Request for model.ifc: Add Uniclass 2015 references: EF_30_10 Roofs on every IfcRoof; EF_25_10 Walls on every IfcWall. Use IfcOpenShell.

First a look at what the model holds.

```python
import ifcopenshell

model = ifcopenshell.open("model.ifc")
print(model.schema)
print("classifications:", [c.Name for c in model.by_type("IfcClassification")])
for ifc_class in ("IfcDoor", "IfcRoof", "IfcStair", "IfcWall", "IfcWindow"):
    print(ifc_class, len(model.by_type(ifc_class)))
```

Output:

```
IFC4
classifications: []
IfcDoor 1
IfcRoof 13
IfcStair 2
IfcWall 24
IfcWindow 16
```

```python
import ifcopenshell
import ifcopenshell.api.classification

model = ifcopenshell.open("model.ifc")

system = ifcopenshell.api.classification.add_classification(model, classification="Uniclass 2015")

codes = {
    "IfcRoof": ("EF_30_10", "Roofs"),
    "IfcWall": ("EF_25_10", "Walls"),
}
for ifc_class, (code, name) in codes.items():
    products = model.by_type(ifc_class)
    ifcopenshell.api.classification.add_reference(
        model, products=products, classification=system, identification=code, name=name
    )
    print(code, len(products))

model.write("model-out.ifc")
```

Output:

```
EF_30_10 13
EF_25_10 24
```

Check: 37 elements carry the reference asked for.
